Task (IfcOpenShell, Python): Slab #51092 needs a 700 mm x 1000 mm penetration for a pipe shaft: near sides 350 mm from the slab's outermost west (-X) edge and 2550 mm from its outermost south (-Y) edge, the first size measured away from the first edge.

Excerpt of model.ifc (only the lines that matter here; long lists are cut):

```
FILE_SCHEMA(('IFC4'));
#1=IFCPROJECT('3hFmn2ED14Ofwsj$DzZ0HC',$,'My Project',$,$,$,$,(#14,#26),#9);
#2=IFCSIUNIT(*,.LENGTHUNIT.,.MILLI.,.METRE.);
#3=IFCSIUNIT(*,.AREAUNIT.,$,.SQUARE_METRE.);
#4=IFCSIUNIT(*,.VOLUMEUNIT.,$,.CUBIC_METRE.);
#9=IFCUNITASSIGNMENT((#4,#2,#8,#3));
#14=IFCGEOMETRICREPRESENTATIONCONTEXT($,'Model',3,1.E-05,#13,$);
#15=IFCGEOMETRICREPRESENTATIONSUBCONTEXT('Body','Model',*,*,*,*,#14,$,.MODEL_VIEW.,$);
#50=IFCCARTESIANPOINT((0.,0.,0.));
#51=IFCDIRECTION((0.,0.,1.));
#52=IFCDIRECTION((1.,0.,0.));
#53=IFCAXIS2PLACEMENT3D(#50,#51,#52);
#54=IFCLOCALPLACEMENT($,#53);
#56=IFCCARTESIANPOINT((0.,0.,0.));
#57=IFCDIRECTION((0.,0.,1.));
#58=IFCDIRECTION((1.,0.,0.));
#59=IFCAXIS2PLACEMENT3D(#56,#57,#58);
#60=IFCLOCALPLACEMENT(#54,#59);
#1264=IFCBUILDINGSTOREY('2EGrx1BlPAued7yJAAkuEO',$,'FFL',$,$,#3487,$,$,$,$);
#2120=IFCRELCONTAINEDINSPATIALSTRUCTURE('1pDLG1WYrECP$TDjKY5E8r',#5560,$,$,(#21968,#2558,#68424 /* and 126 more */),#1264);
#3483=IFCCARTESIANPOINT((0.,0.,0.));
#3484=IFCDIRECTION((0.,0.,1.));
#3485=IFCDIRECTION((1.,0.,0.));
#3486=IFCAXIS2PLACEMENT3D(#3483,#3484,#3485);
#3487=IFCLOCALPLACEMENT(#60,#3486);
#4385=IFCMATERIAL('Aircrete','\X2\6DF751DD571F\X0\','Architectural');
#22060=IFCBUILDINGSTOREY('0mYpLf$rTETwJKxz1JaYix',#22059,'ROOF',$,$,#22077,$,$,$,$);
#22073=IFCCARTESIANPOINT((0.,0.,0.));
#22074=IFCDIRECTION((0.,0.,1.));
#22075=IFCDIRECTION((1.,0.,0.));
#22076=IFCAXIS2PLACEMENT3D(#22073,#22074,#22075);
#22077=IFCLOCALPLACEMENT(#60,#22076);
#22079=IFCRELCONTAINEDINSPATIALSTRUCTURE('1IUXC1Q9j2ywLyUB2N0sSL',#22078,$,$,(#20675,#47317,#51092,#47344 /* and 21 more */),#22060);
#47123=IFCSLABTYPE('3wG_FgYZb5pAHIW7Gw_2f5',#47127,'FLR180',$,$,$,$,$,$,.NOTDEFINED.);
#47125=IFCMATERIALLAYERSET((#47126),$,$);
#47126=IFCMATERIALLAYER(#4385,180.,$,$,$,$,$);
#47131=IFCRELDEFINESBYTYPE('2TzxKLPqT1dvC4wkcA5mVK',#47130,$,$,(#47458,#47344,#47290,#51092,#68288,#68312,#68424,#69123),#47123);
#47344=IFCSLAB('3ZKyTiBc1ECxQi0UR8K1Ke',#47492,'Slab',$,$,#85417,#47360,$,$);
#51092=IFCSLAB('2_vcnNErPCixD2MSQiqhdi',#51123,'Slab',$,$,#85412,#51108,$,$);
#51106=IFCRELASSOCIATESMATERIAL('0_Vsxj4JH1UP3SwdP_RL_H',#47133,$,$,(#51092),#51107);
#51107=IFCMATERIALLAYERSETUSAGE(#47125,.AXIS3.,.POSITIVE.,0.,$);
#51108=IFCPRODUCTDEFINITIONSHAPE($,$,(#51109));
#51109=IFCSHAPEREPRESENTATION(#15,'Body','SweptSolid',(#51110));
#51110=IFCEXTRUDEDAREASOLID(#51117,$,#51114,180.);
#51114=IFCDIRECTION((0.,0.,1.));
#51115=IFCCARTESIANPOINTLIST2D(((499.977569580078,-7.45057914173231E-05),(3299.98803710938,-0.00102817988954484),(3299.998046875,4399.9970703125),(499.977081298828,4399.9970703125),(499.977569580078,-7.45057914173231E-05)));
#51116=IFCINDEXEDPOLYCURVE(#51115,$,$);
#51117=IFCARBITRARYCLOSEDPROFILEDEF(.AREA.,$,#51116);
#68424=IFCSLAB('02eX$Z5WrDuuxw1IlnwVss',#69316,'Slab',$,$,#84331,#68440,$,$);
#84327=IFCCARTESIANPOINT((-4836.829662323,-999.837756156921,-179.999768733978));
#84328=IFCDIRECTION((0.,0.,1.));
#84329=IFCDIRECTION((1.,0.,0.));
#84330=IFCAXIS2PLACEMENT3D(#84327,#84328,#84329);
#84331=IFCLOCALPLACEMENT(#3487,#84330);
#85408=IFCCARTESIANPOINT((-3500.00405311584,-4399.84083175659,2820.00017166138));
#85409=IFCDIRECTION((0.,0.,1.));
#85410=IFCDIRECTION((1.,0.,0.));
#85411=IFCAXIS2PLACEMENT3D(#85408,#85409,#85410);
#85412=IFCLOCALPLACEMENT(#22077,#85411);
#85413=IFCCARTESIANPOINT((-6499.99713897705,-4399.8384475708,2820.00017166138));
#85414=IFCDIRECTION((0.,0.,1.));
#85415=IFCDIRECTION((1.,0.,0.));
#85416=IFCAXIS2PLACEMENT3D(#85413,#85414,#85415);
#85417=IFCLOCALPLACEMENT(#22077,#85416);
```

```python
import numpy as np
import ifcopenshell
import ifcopenshell.api.feature
import ifcopenshell.api.geometry
import ifcopenshell.api.root
import ifcopenshell.geom
import ifcopenshell.util.placement
import ifcopenshell.util.representation
import ifcopenshell.util.shape
import ifcopenshell.util.unit

model = ifcopenshell.open("model.ifc")
unit_scale = ifcopenshell.util.unit.calculate_unit_scale(model)
settings = ifcopenshell.geom.settings()


def volume(element):
    """Net volume in cubic metres, openings subtracted."""
    shape = ifcopenshell.geom.create_shape(settings, element)
    return ifcopenshell.util.shape.get_volume(shape.geometry)


slab = model.by_guid("2_vcnNErPCixD2MSQiqhdi")
before = volume(slab)

# Extent in the slab's own axes, in metres. The edges named are its -X and -Y sides.
slab_shape = ifcopenshell.geom.create_shape(settings, slab)
vertices = ifcopenshell.util.shape.get_vertices(slab_shape.geometry)
x_min, y_min, bottom = vertices.min(axis=0)
top = vertices[:, 2].max()

opening = ifcopenshell.api.root.create_entity(model, ifc_class="IfcOpeningElement", name="Pipe shaft opening", predefined_type="OPENING")
context = ifcopenshell.util.representation.get_context(model, "Model", "Body", "MODEL_VIEW")
width, depth = 0.7, 1
outline = [(0.0, 0.0), (width, 0.0), (width, depth), (0.0, depth), (0.0, 0.0)]
# Overshoot both faces by 50 mm so the cut is clean.
shape = ifcopenshell.api.geometry.add_slab_representation(
    model, context=context, depth=top - bottom + 0.1, polyline=outline
)
ifcopenshell.api.geometry.assign_representation(model, product=opening, representation=shape)

matrix = ifcopenshell.util.placement.get_local_placement(slab.ObjectPlacement)
matrix[:, 3] = matrix @ np.append(np.array([x_min + 0.35, y_min + 2.55, bottom - 0.05]) / unit_scale, 1.0)
ifcopenshell.api.geometry.edit_object_placement(model, product=opening, matrix=matrix, is_si=False)
ifcopenshell.api.feature.add_feature(model, feature=opening, element=slab)

after = volume(slab)

print(f"slab volume {before:.3f} -> {after:.3f} m3")

model.write("model-out.ifc")
```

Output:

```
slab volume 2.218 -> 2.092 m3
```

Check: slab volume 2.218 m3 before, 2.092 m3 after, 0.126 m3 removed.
